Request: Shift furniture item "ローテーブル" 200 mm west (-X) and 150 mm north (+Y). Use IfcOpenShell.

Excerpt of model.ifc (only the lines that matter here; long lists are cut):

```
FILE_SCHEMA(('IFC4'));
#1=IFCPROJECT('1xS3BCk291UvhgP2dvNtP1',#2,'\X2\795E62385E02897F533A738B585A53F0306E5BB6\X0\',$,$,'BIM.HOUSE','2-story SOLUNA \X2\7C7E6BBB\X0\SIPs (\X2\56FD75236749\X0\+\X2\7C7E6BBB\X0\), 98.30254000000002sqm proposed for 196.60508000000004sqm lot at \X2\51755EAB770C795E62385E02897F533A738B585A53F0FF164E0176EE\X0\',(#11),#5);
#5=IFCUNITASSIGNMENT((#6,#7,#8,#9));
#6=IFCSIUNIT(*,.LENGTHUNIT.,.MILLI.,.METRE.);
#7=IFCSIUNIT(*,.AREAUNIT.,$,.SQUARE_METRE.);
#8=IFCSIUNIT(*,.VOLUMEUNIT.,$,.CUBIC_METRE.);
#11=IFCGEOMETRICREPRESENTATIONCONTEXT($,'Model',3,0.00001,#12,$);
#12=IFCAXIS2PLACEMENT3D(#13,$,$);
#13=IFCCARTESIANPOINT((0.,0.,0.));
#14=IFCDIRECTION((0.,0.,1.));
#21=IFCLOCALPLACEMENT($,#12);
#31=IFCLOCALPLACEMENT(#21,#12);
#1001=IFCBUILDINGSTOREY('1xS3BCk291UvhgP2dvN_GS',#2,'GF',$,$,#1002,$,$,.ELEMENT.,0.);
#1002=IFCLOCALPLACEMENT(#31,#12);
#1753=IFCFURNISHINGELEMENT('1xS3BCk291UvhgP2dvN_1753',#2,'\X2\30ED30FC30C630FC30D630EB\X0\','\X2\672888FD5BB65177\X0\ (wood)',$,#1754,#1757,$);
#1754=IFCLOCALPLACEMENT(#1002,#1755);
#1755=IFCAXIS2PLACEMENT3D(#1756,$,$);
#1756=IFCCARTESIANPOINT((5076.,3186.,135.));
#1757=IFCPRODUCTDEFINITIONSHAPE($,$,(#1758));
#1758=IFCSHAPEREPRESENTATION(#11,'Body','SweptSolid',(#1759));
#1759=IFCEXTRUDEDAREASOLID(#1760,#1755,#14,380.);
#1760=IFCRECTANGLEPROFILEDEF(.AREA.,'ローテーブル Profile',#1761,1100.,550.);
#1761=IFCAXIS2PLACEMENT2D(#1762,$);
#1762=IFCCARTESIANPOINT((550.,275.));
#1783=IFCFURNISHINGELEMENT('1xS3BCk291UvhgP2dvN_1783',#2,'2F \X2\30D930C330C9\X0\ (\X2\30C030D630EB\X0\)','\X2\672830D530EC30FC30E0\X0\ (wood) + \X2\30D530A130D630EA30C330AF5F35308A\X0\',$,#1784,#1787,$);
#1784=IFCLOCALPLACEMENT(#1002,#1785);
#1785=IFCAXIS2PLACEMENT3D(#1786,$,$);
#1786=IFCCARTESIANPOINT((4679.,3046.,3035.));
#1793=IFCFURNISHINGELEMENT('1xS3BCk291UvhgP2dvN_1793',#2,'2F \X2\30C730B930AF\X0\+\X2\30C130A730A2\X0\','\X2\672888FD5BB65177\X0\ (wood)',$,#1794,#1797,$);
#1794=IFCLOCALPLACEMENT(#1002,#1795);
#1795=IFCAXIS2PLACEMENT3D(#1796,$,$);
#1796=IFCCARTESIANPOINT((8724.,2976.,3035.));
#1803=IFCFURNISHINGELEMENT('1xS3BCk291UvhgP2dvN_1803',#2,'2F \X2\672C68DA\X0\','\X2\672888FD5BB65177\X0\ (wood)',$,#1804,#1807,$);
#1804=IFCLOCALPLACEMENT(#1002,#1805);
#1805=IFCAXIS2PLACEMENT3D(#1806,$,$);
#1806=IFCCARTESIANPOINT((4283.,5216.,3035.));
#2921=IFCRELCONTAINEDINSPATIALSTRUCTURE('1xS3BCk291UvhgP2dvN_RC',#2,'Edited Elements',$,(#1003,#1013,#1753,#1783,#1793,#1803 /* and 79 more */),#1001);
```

```python
import ifcopenshell
import ifcopenshell.api.geometry
import ifcopenshell.util.placement

model = ifcopenshell.open("model.ifc")

item = model.by_guid("1xS3BCk291UvhgP2dvN_1753")
matrix = ifcopenshell.util.placement.get_local_placement(item.ObjectPlacement)
matrix[0, 3] -= 200.0
matrix[1, 3] += 150.0
ifcopenshell.api.geometry.edit_object_placement(model, product=item, matrix=matrix, is_si=False)

print(ifcopenshell.util.placement.get_local_placement(item.ObjectPlacement).round(3) + 0.0)

model.write("model-out.ifc")
```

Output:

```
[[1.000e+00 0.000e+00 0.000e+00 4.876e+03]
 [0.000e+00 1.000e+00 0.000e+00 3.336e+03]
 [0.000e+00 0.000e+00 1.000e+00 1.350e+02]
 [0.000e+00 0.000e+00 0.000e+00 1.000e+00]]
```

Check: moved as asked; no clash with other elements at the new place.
